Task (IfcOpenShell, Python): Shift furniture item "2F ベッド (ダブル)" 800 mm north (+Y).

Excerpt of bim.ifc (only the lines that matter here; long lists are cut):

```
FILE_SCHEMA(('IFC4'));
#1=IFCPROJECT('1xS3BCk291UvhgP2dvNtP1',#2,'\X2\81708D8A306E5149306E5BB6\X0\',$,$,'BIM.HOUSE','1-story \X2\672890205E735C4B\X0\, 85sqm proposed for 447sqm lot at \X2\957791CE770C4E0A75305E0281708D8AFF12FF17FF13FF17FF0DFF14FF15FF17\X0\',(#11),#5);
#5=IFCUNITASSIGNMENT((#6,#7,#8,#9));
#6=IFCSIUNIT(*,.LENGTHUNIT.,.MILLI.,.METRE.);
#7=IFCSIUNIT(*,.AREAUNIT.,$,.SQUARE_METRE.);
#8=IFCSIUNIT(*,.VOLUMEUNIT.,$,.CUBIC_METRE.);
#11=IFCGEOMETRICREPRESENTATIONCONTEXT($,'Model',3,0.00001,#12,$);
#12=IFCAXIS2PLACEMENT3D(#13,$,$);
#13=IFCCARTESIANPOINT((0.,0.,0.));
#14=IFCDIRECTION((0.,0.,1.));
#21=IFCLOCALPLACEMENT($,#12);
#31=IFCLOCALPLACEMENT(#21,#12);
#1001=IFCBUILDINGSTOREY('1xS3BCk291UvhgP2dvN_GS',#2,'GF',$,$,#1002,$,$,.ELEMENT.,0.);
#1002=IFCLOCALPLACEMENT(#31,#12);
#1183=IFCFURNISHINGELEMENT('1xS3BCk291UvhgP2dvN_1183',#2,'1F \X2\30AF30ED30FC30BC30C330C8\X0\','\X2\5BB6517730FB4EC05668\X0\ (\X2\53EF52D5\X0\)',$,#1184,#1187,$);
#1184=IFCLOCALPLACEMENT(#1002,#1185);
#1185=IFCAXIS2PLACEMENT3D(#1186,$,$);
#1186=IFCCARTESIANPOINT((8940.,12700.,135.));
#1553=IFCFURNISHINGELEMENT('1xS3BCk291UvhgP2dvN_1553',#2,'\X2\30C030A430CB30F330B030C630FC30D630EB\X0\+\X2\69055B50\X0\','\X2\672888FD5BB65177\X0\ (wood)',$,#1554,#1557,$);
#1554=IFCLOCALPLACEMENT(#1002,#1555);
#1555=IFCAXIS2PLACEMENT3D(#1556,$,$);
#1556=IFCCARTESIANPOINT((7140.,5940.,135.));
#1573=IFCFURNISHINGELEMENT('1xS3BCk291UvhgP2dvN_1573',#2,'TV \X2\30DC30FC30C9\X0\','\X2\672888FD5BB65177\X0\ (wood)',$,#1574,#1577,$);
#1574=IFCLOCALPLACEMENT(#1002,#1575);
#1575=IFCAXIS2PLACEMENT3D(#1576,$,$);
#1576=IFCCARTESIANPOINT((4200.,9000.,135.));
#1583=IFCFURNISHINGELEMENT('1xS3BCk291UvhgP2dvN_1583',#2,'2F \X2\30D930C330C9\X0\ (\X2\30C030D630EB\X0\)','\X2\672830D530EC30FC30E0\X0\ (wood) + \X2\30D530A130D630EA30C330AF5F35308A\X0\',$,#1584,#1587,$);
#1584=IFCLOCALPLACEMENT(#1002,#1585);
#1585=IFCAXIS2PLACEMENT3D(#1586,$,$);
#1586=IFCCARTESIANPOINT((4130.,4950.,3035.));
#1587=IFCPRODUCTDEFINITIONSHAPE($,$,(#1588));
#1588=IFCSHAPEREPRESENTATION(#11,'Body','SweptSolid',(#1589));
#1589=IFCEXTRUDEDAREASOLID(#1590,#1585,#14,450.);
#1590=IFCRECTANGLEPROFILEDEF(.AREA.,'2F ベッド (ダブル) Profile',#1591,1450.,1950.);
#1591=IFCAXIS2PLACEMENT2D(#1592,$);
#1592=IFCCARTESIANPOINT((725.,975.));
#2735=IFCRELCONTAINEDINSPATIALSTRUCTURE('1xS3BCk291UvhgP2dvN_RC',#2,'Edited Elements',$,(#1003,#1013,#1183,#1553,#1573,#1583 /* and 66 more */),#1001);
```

```python
import ifcopenshell
import ifcopenshell.api.geometry
import ifcopenshell.util.placement
import ifcopenshell.util.unit

model = ifcopenshell.open("bim.ifc")
unit_scale = ifcopenshell.util.unit.calculate_unit_scale(model)

item = model.by_guid("1xS3BCk291UvhgP2dvN_1583")
matrix = ifcopenshell.util.placement.get_local_placement(item.ObjectPlacement)
matrix[1, 3] += 0.8 / unit_scale
ifcopenshell.api.geometry.edit_object_placement(model, product=item, matrix=matrix, is_si=False)

print(ifcopenshell.util.placement.get_local_placement(item.ObjectPlacement).round(3) + 0.0)

model.write("bim-out.ifc")
```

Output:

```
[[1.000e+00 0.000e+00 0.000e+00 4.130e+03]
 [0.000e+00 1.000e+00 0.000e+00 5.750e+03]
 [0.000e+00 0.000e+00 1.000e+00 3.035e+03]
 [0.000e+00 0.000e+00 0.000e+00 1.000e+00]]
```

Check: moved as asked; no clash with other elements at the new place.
